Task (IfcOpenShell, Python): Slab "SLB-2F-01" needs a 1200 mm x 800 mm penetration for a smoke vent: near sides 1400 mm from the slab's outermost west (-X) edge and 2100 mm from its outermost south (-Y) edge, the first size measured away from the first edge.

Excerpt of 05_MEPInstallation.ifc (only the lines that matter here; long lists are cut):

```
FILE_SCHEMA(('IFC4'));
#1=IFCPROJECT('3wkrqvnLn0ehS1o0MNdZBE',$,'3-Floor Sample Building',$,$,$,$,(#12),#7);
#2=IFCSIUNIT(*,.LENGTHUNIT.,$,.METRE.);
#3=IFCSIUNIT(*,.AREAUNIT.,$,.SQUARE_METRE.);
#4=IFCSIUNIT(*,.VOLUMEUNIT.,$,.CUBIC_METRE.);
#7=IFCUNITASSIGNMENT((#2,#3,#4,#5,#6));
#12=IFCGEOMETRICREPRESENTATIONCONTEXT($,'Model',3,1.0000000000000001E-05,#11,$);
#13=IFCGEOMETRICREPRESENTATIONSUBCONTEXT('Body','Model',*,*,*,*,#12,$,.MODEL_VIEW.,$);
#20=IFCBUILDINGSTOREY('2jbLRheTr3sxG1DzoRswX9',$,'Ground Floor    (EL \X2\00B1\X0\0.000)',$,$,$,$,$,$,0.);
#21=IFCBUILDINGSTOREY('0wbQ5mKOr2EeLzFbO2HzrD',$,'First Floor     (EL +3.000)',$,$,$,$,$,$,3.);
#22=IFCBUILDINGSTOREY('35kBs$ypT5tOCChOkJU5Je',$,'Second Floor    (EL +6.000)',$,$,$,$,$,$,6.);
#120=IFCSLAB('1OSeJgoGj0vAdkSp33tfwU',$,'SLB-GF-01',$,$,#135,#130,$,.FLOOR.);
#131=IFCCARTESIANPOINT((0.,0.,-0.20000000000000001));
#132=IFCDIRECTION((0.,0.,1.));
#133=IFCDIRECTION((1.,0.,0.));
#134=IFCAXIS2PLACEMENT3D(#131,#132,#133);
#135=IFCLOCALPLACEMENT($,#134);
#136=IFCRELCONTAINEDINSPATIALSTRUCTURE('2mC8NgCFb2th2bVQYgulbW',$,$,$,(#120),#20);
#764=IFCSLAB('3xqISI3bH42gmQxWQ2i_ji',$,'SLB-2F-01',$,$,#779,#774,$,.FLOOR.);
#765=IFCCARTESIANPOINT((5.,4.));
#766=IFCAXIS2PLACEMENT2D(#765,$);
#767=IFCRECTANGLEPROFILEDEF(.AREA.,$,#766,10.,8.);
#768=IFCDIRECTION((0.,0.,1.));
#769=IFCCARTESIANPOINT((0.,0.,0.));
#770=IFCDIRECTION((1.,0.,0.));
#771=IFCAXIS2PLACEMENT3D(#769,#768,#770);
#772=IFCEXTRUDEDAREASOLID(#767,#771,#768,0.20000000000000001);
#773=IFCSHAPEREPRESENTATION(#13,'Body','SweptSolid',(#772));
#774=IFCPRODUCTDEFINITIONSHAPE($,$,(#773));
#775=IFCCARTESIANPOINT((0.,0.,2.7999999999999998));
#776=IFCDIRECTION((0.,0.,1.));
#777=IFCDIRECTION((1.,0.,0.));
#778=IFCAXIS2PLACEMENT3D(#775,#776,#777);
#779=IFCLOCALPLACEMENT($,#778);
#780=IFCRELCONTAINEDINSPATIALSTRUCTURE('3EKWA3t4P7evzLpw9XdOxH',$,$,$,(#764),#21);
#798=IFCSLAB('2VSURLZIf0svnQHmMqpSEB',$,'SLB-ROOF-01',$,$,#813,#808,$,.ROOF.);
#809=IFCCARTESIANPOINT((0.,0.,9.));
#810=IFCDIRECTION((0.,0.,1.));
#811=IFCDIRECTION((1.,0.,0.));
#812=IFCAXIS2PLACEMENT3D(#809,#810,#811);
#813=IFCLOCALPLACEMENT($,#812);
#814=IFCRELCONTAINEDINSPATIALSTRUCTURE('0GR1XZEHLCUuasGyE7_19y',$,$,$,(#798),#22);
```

```python
import numpy as np
import ifcopenshell
import ifcopenshell.api.feature
import ifcopenshell.api.geometry
import ifcopenshell.api.root
import ifcopenshell.geom
import ifcopenshell.util.placement
import ifcopenshell.util.representation
import ifcopenshell.util.shape
import ifcopenshell.util.unit

model = ifcopenshell.open("05_MEPInstallation.ifc")
unit_scale = ifcopenshell.util.unit.calculate_unit_scale(model)
settings = ifcopenshell.geom.settings()


def volume(element):
    """Net volume in cubic metres, openings subtracted."""
    shape = ifcopenshell.geom.create_shape(settings, element)
    return ifcopenshell.util.shape.get_volume(shape.geometry)


slab = model.by_guid("3xqISI3bH42gmQxWQ2i_ji")
before = volume(slab)

# Extent in the slab's own axes, in metres. The edges named are its -X and -Y sides.
slab_shape = ifcopenshell.geom.create_shape(settings, slab)
vertices = ifcopenshell.util.shape.get_vertices(slab_shape.geometry)
x_min, y_min, bottom = vertices.min(axis=0)
top = vertices[:, 2].max()

opening = ifcopenshell.api.root.create_entity(model, ifc_class="IfcOpeningElement", name="Smoke vent opening", predefined_type="OPENING")
context = ifcopenshell.util.representation.get_context(model, "Model", "Body", "MODEL_VIEW")
width, depth = 1.2, 0.8
outline = [(0.0, 0.0), (width, 0.0), (width, depth), (0.0, depth), (0.0, 0.0)]
# Overshoot both faces by 50 mm so the cut is clean.
shape = ifcopenshell.api.geometry.add_slab_representation(
    model, context=context, depth=top - bottom + 0.1, polyline=outline
)
ifcopenshell.api.geometry.assign_representation(model, product=opening, representation=shape)

matrix = ifcopenshell.util.placement.get_local_placement(slab.ObjectPlacement)
matrix[:, 3] = matrix @ np.append(np.array([x_min + 1.4, y_min + 2.1, bottom - 0.05]) / unit_scale, 1.0)
ifcopenshell.api.geometry.edit_object_placement(model, product=opening, matrix=matrix, is_si=False)
ifcopenshell.api.feature.add_feature(model, feature=opening, element=slab)

after = volume(slab)

print(f"slab volume {before:.3f} -> {after:.3f} m3")

model.write("05_MEPInstallation_v2.ifc")
```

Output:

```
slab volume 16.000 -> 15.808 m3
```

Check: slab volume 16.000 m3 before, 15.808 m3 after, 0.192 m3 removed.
